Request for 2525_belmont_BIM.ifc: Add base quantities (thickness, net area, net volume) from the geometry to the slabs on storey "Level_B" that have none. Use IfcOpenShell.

First a look at what the model holds.

```python
import ifcopenshell
import ifcopenshell.util.element
import ifcopenshell.util.unit

model = ifcopenshell.open("2525_belmont_BIM.ifc")
print(model.schema)
for unit_type in ("LENGTHUNIT", "AREAUNIT", "VOLUMEUNIT"):
    print(unit_type, ifcopenshell.util.unit.calculate_unit_scale(model, unit_type))
storey = next(s for s in model.by_type("IfcBuildingStorey") if s.Name == "Level_B")
slabs = [e for e in ifcopenshell.util.element.get_decomposition(storey) if e.is_a("IfcSlab")]
for e in sorted(slabs, key=lambda e: e.id()):
    print(e.id(), e.is_a(), e.Name, list(ifcopenshell.util.element.get_psets(e, qtos_only=True)), sep=" | ")
```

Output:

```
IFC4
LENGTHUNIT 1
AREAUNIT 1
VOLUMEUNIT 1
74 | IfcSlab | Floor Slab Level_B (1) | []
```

```python
import ifcopenshell
import ifcopenshell.api.pset
import ifcopenshell.geom
import ifcopenshell.util.element
import ifcopenshell.util.shape
import ifcopenshell.util.unit

model = ifcopenshell.open("2525_belmont_BIM.ifc")
unit_scale = ifcopenshell.util.unit.calculate_unit_scale(model)
area_scale = ifcopenshell.util.unit.calculate_unit_scale(model, "AREAUNIT")
volume_scale = ifcopenshell.util.unit.calculate_unit_scale(model, "VOLUMEUNIT")
settings = ifcopenshell.geom.settings()

storey = next(s for s in model.by_type("IfcBuildingStorey") if s.Name == "Level_B")
slabs = [e for e in ifcopenshell.util.element.get_decomposition(storey) if e.is_a("IfcSlab")]

for e in sorted(slabs, key=lambda e: e.id()):
    if ifcopenshell.util.element.get_psets(e, qtos_only=True, should_inherit=False):
        continue
    # Geometry comes back in metres, in the element's own axes.
    shape = ifcopenshell.geom.create_shape(settings, e)
    values = {
        "Width": ifcopenshell.util.shape.get_z(shape.geometry) / unit_scale,
        "NetArea": ifcopenshell.util.shape.get_footprint_area(shape.geometry) / area_scale,
        "NetVolume": ifcopenshell.util.shape.get_volume(shape.geometry) / volume_scale,
    }
    qto = ifcopenshell.api.pset.add_qto(model, product=e, name="Qto_SlabBaseQuantities")
    ifcopenshell.api.pset.edit_qto(model, qto=qto, properties=values)
    print(e.id(), {k: round(v, 3) for k, v in values.items()})

model.write("2525_belmont_BIM_updated.ifc")
```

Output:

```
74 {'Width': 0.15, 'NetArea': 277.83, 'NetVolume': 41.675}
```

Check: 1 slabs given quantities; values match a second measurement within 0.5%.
